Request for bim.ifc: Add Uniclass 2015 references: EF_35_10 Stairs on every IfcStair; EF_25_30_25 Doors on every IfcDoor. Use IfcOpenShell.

First a look at what the model holds.

```python
import ifcopenshell

model = ifcopenshell.open("bim.ifc")
print(model.schema)
print("classifications:", [c.Name for c in model.by_type("IfcClassification")])
for ifc_class in ("IfcDoor", "IfcRoof", "IfcStair", "IfcWall", "IfcWindow"):
    print(ifc_class, len(model.by_type(ifc_class)))
```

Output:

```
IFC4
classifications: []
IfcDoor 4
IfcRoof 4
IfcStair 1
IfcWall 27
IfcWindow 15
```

```python
import ifcopenshell
import ifcopenshell.api.classification

model = ifcopenshell.open("bim.ifc")

system = ifcopenshell.api.classification.add_classification(model, classification="Uniclass 2015")

codes = {
    "IfcStair": ("EF_35_10", "Stairs"),
    "IfcDoor": ("EF_25_30_25", "Doors"),
}
for ifc_class, (code, name) in codes.items():
    products = model.by_type(ifc_class)
    ifcopenshell.api.classification.add_reference(
        model, products=products, classification=system, identification=code, name=name
    )
    print(code, len(products))

model.write("bim_v2.ifc")
```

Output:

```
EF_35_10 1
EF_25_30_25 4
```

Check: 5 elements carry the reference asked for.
